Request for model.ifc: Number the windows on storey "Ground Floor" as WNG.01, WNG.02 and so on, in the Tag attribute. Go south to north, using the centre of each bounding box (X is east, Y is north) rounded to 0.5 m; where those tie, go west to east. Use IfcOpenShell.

First a look at what the model holds.

```python
import ifcopenshell
import ifcopenshell.util.element
import ifcopenshell.util.placement

model = ifcopenshell.open("model.ifc")
print(model.schema)
storey = next(s for s in model.by_type("IfcBuildingStorey") if s.Name == "Ground Floor")
windows = [e for e in ifcopenshell.util.element.get_decomposition(storey) if e.is_a("IfcWindow")]
for e in sorted(windows, key=lambda e: e.id()):
    origin = ifcopenshell.util.placement.get_local_placement(e.ObjectPlacement)[:3, 3]
    print(e.id(), e.Tag, e.Name, origin.round(2) + 0.0, sep=" | ")
```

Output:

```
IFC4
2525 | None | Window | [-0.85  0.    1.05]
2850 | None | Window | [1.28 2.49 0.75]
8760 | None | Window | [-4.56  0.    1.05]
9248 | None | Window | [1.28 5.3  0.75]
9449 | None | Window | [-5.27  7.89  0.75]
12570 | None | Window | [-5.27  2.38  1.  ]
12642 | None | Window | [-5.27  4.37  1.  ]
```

```python
import ifcopenshell
import ifcopenshell.geom
import ifcopenshell.util.element
import ifcopenshell.util.shape

model = ifcopenshell.open("model.ifc")
settings = ifcopenshell.geom.settings()
settings.set("use-world-coords", True)


def centre(element):
    shape = ifcopenshell.geom.create_shape(settings, element)
    return ifcopenshell.util.shape.get_bbox_centroid(shape.geometry)


storey = next(s for s in model.by_type("IfcBuildingStorey") if s.Name == "Ground Floor")
windows = [e for e in ifcopenshell.util.element.get_decomposition(storey) if e.is_a("IfcWindow")]

# Insertion points can sit at a corner or the storey origin, so sort by the geometry (in metres).
centres = {e: centre(e) for e in windows}
windows.sort(key=lambda e: (round(centres[e][1] / 0.5), centres[e][0]))

for i, e in enumerate(windows, start=1):
    number = f"WNG.{i:02d}"
    e.Tag = number
    print(e.id(), number)

model.write("model_rev.ifc")
```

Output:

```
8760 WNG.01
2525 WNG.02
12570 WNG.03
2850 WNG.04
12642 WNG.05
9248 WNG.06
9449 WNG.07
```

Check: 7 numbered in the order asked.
